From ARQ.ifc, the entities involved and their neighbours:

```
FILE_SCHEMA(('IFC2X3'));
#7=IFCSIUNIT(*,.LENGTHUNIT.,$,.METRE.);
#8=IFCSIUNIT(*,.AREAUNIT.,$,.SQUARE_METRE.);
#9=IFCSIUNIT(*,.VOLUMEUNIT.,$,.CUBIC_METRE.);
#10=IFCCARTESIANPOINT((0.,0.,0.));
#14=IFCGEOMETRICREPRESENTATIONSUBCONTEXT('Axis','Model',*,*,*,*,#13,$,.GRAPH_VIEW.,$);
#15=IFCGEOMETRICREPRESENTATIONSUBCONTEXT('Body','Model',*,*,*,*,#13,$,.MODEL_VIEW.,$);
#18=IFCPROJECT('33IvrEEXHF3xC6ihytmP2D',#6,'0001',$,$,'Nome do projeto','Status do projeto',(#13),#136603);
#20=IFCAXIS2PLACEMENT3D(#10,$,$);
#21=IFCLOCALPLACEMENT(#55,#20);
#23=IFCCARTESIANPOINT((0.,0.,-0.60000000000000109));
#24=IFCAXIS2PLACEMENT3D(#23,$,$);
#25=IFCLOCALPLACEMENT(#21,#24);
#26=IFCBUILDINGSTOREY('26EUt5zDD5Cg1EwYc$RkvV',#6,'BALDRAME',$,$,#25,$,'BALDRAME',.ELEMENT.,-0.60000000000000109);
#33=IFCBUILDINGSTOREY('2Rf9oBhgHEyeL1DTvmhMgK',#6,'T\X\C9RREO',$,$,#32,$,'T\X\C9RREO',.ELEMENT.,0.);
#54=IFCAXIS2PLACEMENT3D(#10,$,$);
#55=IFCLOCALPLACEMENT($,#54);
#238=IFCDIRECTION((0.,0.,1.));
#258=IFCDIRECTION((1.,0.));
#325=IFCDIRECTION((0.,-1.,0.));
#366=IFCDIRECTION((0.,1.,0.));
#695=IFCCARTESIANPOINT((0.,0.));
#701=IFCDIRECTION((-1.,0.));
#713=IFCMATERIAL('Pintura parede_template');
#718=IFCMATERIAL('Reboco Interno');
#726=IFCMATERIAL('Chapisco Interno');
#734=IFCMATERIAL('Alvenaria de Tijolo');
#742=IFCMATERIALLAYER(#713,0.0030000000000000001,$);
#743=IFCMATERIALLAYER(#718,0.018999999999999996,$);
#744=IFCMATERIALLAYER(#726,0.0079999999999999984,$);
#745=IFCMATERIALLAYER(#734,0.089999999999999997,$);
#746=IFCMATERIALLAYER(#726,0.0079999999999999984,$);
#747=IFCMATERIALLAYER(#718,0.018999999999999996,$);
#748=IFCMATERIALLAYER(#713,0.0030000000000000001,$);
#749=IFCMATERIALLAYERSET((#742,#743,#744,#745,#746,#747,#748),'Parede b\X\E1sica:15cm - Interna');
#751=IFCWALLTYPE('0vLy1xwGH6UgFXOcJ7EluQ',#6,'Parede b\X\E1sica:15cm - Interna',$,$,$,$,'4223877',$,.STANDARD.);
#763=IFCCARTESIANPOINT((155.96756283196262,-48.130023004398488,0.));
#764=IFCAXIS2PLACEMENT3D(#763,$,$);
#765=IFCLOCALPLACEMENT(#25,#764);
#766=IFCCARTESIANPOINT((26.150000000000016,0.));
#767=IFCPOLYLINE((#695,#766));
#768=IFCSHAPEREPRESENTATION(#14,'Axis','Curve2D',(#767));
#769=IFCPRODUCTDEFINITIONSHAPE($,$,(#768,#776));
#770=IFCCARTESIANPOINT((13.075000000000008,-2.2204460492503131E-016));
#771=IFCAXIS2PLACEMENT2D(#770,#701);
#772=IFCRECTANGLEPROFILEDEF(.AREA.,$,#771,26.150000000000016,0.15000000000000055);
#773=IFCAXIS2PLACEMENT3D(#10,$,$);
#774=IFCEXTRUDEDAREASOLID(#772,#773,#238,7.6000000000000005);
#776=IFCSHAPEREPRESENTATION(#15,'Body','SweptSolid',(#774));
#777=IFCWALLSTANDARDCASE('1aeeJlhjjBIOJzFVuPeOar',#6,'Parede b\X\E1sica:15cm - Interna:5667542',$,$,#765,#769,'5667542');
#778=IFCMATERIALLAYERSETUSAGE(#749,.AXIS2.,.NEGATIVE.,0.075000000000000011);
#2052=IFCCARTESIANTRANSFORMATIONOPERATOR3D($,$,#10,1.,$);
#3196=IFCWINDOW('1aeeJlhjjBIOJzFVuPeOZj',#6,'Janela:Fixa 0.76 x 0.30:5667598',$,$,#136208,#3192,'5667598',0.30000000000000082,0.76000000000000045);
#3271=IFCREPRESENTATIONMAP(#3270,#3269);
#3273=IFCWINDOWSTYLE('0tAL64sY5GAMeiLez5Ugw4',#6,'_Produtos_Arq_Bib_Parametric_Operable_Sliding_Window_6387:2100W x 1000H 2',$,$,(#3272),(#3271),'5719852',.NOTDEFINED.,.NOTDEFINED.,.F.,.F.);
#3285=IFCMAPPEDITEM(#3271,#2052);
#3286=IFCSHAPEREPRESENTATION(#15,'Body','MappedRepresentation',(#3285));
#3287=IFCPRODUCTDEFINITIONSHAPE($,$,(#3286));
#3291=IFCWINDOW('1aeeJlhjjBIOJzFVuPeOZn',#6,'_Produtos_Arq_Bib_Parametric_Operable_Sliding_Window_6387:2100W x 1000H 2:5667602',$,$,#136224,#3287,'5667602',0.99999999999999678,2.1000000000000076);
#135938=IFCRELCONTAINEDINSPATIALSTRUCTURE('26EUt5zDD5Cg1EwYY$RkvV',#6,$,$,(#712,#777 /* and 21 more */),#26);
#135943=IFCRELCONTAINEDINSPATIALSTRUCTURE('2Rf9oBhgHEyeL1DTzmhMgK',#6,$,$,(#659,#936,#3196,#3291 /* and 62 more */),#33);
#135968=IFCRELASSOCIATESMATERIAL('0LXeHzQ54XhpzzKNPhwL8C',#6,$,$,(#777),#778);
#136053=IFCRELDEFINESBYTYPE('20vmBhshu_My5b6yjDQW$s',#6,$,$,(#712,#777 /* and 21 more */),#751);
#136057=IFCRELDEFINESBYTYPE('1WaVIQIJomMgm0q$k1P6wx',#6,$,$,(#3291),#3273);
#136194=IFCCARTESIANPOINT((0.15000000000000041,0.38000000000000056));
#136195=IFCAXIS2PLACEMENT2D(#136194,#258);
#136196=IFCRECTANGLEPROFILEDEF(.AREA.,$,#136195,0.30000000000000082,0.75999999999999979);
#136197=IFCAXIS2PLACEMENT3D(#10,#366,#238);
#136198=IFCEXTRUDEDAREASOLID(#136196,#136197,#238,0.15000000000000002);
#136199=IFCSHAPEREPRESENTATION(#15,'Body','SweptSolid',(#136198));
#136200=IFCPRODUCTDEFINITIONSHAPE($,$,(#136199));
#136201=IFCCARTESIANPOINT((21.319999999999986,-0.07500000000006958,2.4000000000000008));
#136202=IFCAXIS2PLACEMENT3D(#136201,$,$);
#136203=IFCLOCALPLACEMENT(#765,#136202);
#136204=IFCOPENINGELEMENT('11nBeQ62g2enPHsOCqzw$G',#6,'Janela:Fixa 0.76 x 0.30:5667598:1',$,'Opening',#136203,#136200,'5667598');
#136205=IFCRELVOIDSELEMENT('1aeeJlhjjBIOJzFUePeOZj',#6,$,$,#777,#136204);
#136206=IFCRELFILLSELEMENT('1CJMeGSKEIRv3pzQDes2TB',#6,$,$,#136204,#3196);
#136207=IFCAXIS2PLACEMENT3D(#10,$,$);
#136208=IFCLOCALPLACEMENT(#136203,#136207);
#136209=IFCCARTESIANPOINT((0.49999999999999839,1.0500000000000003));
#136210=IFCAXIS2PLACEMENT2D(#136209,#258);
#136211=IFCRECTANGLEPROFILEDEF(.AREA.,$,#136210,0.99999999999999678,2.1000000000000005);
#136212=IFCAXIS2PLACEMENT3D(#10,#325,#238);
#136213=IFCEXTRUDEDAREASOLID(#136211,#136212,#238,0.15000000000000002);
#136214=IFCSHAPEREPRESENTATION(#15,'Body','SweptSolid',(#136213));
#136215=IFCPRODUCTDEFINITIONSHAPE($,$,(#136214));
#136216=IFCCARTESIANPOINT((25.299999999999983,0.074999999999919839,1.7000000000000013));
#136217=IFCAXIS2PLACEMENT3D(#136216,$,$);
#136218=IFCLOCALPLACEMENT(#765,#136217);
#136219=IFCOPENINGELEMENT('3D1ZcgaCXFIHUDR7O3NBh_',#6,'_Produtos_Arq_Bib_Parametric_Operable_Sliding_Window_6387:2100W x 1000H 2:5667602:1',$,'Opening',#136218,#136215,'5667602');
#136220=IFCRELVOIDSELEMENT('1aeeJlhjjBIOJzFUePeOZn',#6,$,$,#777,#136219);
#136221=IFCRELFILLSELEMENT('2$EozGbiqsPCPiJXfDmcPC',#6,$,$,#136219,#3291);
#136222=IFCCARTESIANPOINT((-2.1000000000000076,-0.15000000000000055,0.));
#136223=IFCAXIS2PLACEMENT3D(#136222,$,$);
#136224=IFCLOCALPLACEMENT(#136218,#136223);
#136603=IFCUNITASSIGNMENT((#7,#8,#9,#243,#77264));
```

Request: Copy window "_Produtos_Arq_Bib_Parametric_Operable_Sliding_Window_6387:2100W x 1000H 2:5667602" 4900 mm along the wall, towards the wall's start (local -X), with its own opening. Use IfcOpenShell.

```python
import ifcopenshell
import ifcopenshell.api.feature
import ifcopenshell.api.geometry
import ifcopenshell.api.root
import ifcopenshell.geom
import ifcopenshell.util.element
import ifcopenshell.util.placement
import ifcopenshell.util.shape
import ifcopenshell.util.unit

model = ifcopenshell.open("ARQ.ifc")
unit_scale = ifcopenshell.util.unit.calculate_unit_scale(model)
settings = ifcopenshell.geom.settings()


def volume(element):
    """Net volume in cubic metres, openings subtracted."""
    shape = ifcopenshell.geom.create_shape(settings, element)
    return ifcopenshell.util.shape.get_volume(shape.geometry)


def reuse_history(source, copy):
    """copy_class also copies each property set's owner history, people and application; keep the originals."""
    for rel in copy.IsDefinedBy:
        if rel.is_a("IfcRelDefinesByProperties") and (history := rel.RelatingPropertyDefinition.OwnerHistory):
            rel.RelatingPropertyDefinition.OwnerHistory = source.OwnerHistory
            ifcopenshell.util.element.remove_deep2(model, history)


window = model.by_id(3291)
opening = window.FillsVoids[0].RelatingOpeningElement
wall = opening.VoidsElements[0].RelatingBuildingElement
before = volume(wall)
shift = ifcopenshell.util.placement.get_local_placement(wall.ObjectPlacement)[:3, 0] * -4.9 / unit_scale

# copy_class copies the void relationship, type, container and properties, but no geometry.
new_opening = ifcopenshell.api.root.copy_class(model, product=opening)
new_opening.Representation = ifcopenshell.util.element.copy_deep(
    model, opening.Representation, exclude=["IfcGeometricRepresentationContext", "IfcRepresentationMap"]
)
new_opening.Name = "_Produtos_Arq_Bib_Parametric_Operable_Sliding_Window_6387:2100W x 1000H 2"
new_opening.Tag = None
new_window = ifcopenshell.api.root.copy_class(model, product=window)
new_window.Representation = ifcopenshell.util.element.copy_deep(
    model, window.Representation, exclude=["IfcGeometricRepresentationContext", "IfcRepresentationMap"]
)
new_window.Name = "_Produtos_Arq_Bib_Parametric_Operable_Sliding_Window_6387:2100W x 1000H 2"
new_window.Tag = None
reuse_history(window, new_window)
fills = ifcopenshell.api.feature.add_filling(model, opening=new_opening, element=new_window)
fills.OwnerHistory = new_window.OwnerHistory  # required in IFC2X3

for old, new in ((opening, new_opening), (window, new_window)):
    matrix = ifcopenshell.util.placement.get_local_placement(old.ObjectPlacement)
    matrix[:3, 3] += shift
    ifcopenshell.api.geometry.edit_object_placement(model, product=new, matrix=matrix, is_si=False)

after = volume(wall)

print(f"wall volume {before:.3f} -> {after:.3f} m3")

model.write("ARQ_edited.ifc")
```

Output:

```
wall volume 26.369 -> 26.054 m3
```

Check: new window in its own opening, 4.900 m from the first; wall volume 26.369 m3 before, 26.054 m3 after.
